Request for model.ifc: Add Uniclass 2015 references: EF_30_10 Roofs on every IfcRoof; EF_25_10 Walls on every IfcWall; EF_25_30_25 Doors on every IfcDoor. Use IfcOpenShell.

First a look at what the model holds.

```python
import ifcopenshell

model = ifcopenshell.open("model.ifc")
print(model.schema)
print("classifications:", [c.Name for c in model.by_type("IfcClassification")])
for ifc_class in ("IfcDoor", "IfcRoof", "IfcStair", "IfcWall", "IfcWindow"):
    print(ifc_class, len(model.by_type(ifc_class)))
```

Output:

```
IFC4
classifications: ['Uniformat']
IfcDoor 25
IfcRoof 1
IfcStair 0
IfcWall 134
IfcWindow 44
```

```python
import ifcopenshell
import ifcopenshell.api.classification

model = ifcopenshell.open("model.ifc")

system = ifcopenshell.api.classification.add_classification(model, classification="Uniclass 2015")

codes = {
    "IfcRoof": ("EF_30_10", "Roofs"),
    "IfcWall": ("EF_25_10", "Walls"),
    "IfcDoor": ("EF_25_30_25", "Doors"),
}
for ifc_class, (code, name) in codes.items():
    products = model.by_type(ifc_class)
    ifcopenshell.api.classification.add_reference(
        model, products=products, classification=system, identification=code, name=name
    )
    print(code, len(products))

model.write("model_edited.ifc")
```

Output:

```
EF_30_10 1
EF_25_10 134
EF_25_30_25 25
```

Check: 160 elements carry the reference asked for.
